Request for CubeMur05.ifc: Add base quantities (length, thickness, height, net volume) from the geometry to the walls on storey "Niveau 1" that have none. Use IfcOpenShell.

First a look at what the model holds.

```python
import ifcopenshell
import ifcopenshell.util.element
import ifcopenshell.util.unit

model = ifcopenshell.open("CubeMur05.ifc")
print(model.schema)
for unit_type in ("LENGTHUNIT", "AREAUNIT", "VOLUMEUNIT"):
    print(unit_type, ifcopenshell.util.unit.calculate_unit_scale(model, unit_type))
storey = next(s for s in model.by_type("IfcBuildingStorey") if s.Name == "Niveau 1")
walls = [e for e in ifcopenshell.util.element.get_decomposition(storey) if e.is_a("IfcWall")]
for e in sorted(walls, key=lambda e: e.id()):
    print(e.id(), e.is_a(), e.Name, list(ifcopenshell.util.element.get_psets(e, qtos_only=True)), sep=" | ")
```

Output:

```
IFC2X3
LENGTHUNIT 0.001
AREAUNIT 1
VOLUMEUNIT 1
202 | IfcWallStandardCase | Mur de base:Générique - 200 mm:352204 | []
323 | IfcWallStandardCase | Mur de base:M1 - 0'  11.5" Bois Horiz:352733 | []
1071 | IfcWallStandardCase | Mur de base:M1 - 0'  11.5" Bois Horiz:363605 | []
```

```python
import ifcopenshell
import ifcopenshell.api.pset
import ifcopenshell.geom
import ifcopenshell.util.element
import ifcopenshell.util.shape
import ifcopenshell.util.unit

model = ifcopenshell.open("CubeMur05.ifc")
unit_scale = ifcopenshell.util.unit.calculate_unit_scale(model)
volume_scale = ifcopenshell.util.unit.calculate_unit_scale(model, "VOLUMEUNIT")
settings = ifcopenshell.geom.settings()

storey = next(s for s in model.by_type("IfcBuildingStorey") if s.Name == "Niveau 1")
walls = [e for e in ifcopenshell.util.element.get_decomposition(storey) if e.is_a("IfcWall")]

for e in sorted(walls, key=lambda e: e.id()):
    if ifcopenshell.util.element.get_psets(e, qtos_only=True, should_inherit=False):
        continue
    # Geometry comes back in metres, in the element's own axes.
    shape = ifcopenshell.geom.create_shape(settings, e)
    values = {
        "Length": ifcopenshell.util.shape.get_x(shape.geometry) / unit_scale,
        "Width": ifcopenshell.util.shape.get_y(shape.geometry) / unit_scale,
        "Height": ifcopenshell.util.shape.get_z(shape.geometry) / unit_scale,
        "NetVolume": ifcopenshell.util.shape.get_volume(shape.geometry) / volume_scale,
    }
    qto = ifcopenshell.api.pset.add_qto(model, product=e, name="BaseQuantities")
    ifcopenshell.api.pset.edit_qto(model, qto=qto, properties=values)
    print(e.id(), {k: round(v, 3) for k, v in values.items()})

model.write("CubeMur05_v2.ifc")
```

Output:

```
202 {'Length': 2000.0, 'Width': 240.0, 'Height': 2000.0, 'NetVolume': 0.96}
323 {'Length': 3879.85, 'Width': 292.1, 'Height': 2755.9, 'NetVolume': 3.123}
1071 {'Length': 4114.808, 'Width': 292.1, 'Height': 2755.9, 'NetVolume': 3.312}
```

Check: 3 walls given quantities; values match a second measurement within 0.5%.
